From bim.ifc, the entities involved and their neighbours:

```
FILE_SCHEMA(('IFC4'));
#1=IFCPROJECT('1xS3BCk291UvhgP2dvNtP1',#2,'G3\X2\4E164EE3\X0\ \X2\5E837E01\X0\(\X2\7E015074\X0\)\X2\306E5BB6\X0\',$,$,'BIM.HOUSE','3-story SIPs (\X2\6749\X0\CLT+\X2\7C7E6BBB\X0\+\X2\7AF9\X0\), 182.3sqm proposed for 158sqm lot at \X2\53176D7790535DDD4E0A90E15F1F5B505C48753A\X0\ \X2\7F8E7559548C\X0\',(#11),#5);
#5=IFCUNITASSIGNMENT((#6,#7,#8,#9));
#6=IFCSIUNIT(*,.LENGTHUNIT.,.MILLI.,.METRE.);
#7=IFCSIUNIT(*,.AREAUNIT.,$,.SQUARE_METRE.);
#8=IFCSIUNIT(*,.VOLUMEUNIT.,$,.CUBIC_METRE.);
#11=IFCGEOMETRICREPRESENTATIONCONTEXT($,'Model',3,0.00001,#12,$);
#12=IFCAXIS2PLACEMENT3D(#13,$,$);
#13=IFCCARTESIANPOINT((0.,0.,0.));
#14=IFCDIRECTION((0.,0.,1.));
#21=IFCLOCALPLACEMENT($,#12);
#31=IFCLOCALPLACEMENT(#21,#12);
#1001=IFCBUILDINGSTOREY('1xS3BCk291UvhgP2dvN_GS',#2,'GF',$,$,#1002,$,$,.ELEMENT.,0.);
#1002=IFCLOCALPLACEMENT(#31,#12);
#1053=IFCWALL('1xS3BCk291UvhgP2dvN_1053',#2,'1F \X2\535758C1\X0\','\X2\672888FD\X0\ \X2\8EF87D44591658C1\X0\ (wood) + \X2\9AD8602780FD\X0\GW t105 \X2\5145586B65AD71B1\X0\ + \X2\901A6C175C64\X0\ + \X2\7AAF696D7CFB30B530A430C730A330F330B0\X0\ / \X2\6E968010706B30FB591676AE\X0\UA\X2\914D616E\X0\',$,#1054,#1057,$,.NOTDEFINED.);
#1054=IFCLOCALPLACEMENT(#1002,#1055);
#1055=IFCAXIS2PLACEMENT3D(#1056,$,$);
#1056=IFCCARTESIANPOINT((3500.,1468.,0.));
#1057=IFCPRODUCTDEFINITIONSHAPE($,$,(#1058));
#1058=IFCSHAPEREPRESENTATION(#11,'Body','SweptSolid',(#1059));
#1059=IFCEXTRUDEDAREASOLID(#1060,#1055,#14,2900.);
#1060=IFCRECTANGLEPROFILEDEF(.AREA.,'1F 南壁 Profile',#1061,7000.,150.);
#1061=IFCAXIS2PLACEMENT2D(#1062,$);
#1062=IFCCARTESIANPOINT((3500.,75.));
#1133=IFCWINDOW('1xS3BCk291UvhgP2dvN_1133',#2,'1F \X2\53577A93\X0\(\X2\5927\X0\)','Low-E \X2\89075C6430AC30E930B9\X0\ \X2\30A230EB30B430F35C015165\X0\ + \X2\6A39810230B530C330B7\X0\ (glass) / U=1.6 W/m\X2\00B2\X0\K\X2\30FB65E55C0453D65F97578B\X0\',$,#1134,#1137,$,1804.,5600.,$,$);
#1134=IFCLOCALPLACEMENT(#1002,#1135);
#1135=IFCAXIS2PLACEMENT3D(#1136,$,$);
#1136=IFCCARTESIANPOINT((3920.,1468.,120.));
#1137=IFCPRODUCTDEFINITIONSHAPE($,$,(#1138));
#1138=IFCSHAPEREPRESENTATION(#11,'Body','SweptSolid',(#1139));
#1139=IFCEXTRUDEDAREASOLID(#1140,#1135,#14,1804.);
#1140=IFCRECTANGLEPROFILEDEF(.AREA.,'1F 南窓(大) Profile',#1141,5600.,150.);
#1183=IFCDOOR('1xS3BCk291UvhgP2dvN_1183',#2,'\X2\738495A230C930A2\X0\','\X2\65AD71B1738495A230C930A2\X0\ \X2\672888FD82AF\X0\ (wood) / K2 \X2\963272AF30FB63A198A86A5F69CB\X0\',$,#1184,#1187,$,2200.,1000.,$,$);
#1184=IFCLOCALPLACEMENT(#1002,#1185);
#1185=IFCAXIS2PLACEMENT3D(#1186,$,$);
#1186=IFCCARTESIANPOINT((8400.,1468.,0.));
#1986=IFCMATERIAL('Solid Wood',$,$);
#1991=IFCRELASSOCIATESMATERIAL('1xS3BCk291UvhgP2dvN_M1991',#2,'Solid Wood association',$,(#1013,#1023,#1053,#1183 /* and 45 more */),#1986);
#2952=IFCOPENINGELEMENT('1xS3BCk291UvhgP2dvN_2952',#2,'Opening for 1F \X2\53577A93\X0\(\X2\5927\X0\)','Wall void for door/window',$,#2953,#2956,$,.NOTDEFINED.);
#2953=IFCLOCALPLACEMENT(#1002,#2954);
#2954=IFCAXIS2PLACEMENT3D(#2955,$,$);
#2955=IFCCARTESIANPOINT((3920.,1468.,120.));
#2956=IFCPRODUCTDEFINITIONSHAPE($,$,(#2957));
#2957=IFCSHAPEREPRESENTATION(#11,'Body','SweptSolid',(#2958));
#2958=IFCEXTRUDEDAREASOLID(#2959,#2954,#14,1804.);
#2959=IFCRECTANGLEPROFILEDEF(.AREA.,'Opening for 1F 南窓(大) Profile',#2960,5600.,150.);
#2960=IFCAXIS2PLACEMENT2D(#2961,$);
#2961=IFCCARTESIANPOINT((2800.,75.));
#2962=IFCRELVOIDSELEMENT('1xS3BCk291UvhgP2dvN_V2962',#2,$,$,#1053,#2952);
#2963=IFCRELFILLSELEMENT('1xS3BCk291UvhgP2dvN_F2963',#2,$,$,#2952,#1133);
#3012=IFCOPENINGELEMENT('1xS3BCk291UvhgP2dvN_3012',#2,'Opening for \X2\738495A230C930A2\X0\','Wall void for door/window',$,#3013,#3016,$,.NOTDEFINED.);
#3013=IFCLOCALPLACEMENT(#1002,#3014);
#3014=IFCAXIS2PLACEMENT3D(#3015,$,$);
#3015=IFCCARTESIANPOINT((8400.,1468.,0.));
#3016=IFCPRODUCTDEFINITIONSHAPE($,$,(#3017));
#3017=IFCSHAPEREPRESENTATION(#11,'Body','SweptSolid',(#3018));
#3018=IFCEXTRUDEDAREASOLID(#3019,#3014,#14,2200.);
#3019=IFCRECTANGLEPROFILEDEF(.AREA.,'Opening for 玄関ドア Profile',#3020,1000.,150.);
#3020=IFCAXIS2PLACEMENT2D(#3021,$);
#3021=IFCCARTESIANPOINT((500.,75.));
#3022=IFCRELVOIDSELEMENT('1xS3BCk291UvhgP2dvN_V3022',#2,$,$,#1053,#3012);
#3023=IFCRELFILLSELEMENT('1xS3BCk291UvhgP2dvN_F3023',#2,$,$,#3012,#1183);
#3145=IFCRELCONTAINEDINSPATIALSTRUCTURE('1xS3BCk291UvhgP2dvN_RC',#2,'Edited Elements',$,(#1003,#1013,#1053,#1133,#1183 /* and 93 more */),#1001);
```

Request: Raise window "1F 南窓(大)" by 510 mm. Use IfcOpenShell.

```python
import numpy as np
import ifcopenshell
import ifcopenshell.api.geometry
import ifcopenshell.util.placement
import ifcopenshell.util.unit

model = ifcopenshell.open("bim.ifc")
unit_scale = ifcopenshell.util.unit.calculate_unit_scale(model)

window = model.by_guid("1xS3BCk291UvhgP2dvN_1133")
opening = window.FillsVoids[0].RelatingOpeningElement
dz = 510.0

shift = np.array([0.0, 0.0, dz])
# The window is not placed relative to its opening, so move both.
for product in (opening, window):
    matrix = ifcopenshell.util.placement.get_local_placement(product.ObjectPlacement)
    matrix[:3, 3] += shift
    ifcopenshell.api.geometry.edit_object_placement(model, product=product, matrix=matrix, is_si=False)

print(f"moved by {dz * unit_scale:+.3f} m")

model.write("bim_updated.ifc")
```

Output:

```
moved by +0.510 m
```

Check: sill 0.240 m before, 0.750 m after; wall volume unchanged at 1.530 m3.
